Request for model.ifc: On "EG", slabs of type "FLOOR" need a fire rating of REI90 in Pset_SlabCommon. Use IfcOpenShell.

First a look at what the model holds.

```python
import ifcopenshell
import ifcopenshell.util.element

model = ifcopenshell.open("model.ifc")
print(model.schema)
storey = next(s for s in model.by_type("IfcBuildingStorey") if s.Name == "EG")
slabs = [e for e in ifcopenshell.util.element.get_decomposition(storey) if e.is_a("IfcSlab")]
seen = {}
for e in slabs:
    element_type = ifcopenshell.util.element.get_type(e)
    key = (element_type.Name if element_type != e and element_type else None, ifcopenshell.util.element.get_pset(e, "Pset_SlabCommon", "FireRating"))
    seen[key] = seen.get(key, 0) + 1
for (name, value), count in sorted(seen.items(), key=str):
    print(count, "x", name, "|", value)
```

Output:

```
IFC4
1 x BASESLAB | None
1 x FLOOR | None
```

```python
import ifcopenshell
import ifcopenshell.api.pset
import ifcopenshell.util.element

model = ifcopenshell.open("model.ifc")

storey = next(s for s in model.by_type("IfcBuildingStorey") if s.Name == "EG")
slabs = [e for e in ifcopenshell.util.element.get_decomposition(storey) if e.is_a("IfcSlab")]

count = 0
for e in slabs:
    element_type = ifcopenshell.util.element.get_type(e)
    if element_type in (None, e) or element_type.Name != "FLOOR":
        continue
    # add_pset returns the element's existing set when there is one.
    pset = ifcopenshell.api.pset.add_pset(model, product=e, name="Pset_SlabCommon")
    ifcopenshell.api.pset.edit_pset(model, pset=pset, properties={"FireRating": "REI90"})
    count += 1

print(count, "slabs updated")

model.write("model_updated.ifc")
```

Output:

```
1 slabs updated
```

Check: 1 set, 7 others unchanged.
